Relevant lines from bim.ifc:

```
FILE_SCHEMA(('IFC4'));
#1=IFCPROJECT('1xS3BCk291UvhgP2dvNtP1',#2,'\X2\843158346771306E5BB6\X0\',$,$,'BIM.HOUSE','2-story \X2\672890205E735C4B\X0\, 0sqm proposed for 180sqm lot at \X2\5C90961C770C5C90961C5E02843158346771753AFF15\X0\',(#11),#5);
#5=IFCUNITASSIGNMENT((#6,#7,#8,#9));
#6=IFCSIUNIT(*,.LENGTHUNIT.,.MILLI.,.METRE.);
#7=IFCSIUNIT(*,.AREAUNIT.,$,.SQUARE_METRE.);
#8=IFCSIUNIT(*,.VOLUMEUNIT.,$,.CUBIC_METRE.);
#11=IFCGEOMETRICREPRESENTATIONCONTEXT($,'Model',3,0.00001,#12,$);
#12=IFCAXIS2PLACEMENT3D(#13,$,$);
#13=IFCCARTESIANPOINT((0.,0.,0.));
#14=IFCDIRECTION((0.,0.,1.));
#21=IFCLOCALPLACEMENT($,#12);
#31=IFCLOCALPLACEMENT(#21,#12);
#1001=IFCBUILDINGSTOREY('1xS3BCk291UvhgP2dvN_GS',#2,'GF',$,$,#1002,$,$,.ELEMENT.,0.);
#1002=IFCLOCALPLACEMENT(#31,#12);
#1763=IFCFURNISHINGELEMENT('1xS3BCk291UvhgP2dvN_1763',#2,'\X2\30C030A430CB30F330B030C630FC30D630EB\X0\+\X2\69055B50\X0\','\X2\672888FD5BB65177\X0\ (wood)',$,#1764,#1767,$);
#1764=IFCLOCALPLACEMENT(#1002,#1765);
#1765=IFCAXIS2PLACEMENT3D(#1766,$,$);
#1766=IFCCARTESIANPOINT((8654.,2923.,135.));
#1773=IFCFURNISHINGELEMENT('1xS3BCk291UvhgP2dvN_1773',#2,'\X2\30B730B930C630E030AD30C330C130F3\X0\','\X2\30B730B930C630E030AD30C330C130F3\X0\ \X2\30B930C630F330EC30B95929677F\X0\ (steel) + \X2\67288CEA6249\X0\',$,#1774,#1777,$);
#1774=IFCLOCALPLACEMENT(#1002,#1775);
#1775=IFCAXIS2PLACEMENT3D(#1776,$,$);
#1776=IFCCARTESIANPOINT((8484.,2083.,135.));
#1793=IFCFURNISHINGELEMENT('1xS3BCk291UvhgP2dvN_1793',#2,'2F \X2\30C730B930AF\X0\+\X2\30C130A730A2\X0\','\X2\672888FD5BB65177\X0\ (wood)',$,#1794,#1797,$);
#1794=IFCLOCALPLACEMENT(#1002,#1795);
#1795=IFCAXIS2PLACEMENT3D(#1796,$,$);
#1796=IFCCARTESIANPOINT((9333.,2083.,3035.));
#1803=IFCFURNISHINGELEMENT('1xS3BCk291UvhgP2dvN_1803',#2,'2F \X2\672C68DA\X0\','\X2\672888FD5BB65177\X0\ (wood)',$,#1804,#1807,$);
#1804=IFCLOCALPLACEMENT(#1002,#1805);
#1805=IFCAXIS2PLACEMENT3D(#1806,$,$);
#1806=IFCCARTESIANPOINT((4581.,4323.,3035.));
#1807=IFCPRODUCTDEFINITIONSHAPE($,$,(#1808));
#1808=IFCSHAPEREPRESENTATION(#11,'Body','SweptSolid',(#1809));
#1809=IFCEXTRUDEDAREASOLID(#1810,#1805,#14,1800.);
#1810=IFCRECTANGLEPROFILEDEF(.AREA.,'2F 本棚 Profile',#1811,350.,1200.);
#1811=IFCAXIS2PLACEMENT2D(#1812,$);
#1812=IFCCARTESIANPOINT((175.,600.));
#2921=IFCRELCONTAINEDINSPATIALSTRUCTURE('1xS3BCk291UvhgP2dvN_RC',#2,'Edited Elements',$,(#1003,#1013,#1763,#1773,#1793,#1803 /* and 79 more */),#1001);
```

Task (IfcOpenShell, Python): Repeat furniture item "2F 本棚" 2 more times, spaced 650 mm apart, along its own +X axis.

```python
import ifcopenshell
import ifcopenshell.api.geometry
import ifcopenshell.api.root
import ifcopenshell.util.element
import ifcopenshell.util.placement
import ifcopenshell.util.unit

model = ifcopenshell.open("bim.ifc")
unit_scale = ifcopenshell.util.unit.calculate_unit_scale(model)


def reuse_history(source, copy):
    """copy_class also copies each property set's owner history, people and application; keep the originals."""
    for rel in copy.IsDefinedBy:
        if rel.is_a("IfcRelDefinesByProperties") and (history := rel.RelatingPropertyDefinition.OwnerHistory):
            rel.RelatingPropertyDefinition.OwnerHistory = source.OwnerHistory
            ifcopenshell.util.element.remove_deep2(model, history)


source = model.by_guid("1xS3BCk291UvhgP2dvN_1803")
base = ifcopenshell.util.placement.get_local_placement(source.ObjectPlacement)
step = base[:3, 0] * 0.65 / unit_scale

for i in range(1, 3):
    copy = ifcopenshell.api.root.copy_class(model, product=source)
    copy.Representation = ifcopenshell.util.element.copy_deep(
        model, source.Representation, exclude=["IfcGeometricRepresentationContext", "IfcRepresentationMap"]
    )
    reuse_history(source, copy)
    matrix = base.copy()
    matrix[:3, 3] += i * step
    print("added at", matrix[:3, 3].round(3) + 0.0)
    ifcopenshell.api.geometry.edit_object_placement(model, product=copy, matrix=matrix, is_si=False)

model.write("bim_rev.ifc")
```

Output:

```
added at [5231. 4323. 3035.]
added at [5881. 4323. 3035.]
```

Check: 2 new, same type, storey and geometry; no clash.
